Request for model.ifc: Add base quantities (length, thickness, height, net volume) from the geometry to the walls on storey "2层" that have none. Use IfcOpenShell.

First a look at what the model holds.

```python
import ifcopenshell
import ifcopenshell.util.element
import ifcopenshell.util.unit

model = ifcopenshell.open("model.ifc")
print(model.schema)
for unit_type in ("LENGTHUNIT", "AREAUNIT", "VOLUMEUNIT"):
    print(unit_type, ifcopenshell.util.unit.calculate_unit_scale(model, unit_type))
storey = next(s for s in model.by_type("IfcBuildingStorey") if s.Name == "2层")
walls = [e for e in ifcopenshell.util.element.get_decomposition(storey) if e.is_a("IfcWall")]
for e in sorted(walls, key=lambda e: e.id()):
    print(e.id(), e.is_a(), e.Name, list(ifcopenshell.util.element.get_psets(e, qtos_only=True)), sep=" | ")
```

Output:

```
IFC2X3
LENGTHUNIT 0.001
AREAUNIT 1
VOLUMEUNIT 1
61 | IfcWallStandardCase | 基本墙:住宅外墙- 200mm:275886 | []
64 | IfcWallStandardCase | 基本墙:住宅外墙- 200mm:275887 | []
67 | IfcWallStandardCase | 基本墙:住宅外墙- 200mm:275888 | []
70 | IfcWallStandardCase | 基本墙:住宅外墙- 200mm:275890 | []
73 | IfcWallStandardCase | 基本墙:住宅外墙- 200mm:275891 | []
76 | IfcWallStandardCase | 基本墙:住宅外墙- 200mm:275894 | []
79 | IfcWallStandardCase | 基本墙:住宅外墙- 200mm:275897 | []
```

```python
import ifcopenshell
import ifcopenshell.api.pset
import ifcopenshell.geom
import ifcopenshell.util.element
import ifcopenshell.util.shape
import ifcopenshell.util.unit

model = ifcopenshell.open("model.ifc")
unit_scale = ifcopenshell.util.unit.calculate_unit_scale(model)
volume_scale = ifcopenshell.util.unit.calculate_unit_scale(model, "VOLUMEUNIT")
settings = ifcopenshell.geom.settings()

storey = next(s for s in model.by_type("IfcBuildingStorey") if s.Name == "2层")
walls = [e for e in ifcopenshell.util.element.get_decomposition(storey) if e.is_a("IfcWall")]

for e in sorted(walls, key=lambda e: e.id()):
    if ifcopenshell.util.element.get_psets(e, qtos_only=True, should_inherit=False):
        continue
    # Geometry comes back in metres, in the element's own axes.
    shape = ifcopenshell.geom.create_shape(settings, e)
    values = {
        "Length": ifcopenshell.util.shape.get_x(shape.geometry) / unit_scale,
        "Width": ifcopenshell.util.shape.get_y(shape.geometry) / unit_scale,
        "Height": ifcopenshell.util.shape.get_z(shape.geometry) / unit_scale,
        "NetVolume": ifcopenshell.util.shape.get_volume(shape.geometry) / volume_scale,
    }
    qto = ifcopenshell.api.pset.add_qto(model, product=e, name="BaseQuantities")
    ifcopenshell.api.pset.edit_qto(model, qto=qto, properties=values)
    print(e.id(), {k: round(v, 3) for k, v in values.items()})

model.write("model_updated.ifc")
```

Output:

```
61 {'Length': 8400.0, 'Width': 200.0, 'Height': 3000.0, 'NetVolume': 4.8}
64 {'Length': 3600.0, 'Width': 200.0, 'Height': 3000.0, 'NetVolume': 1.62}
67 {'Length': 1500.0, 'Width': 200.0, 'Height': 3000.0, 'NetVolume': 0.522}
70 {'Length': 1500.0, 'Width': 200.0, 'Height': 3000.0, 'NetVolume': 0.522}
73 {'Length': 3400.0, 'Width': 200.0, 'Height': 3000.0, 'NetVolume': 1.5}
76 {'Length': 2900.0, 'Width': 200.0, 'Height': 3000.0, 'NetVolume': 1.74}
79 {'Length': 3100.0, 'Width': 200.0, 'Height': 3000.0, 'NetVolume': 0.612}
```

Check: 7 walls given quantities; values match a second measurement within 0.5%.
